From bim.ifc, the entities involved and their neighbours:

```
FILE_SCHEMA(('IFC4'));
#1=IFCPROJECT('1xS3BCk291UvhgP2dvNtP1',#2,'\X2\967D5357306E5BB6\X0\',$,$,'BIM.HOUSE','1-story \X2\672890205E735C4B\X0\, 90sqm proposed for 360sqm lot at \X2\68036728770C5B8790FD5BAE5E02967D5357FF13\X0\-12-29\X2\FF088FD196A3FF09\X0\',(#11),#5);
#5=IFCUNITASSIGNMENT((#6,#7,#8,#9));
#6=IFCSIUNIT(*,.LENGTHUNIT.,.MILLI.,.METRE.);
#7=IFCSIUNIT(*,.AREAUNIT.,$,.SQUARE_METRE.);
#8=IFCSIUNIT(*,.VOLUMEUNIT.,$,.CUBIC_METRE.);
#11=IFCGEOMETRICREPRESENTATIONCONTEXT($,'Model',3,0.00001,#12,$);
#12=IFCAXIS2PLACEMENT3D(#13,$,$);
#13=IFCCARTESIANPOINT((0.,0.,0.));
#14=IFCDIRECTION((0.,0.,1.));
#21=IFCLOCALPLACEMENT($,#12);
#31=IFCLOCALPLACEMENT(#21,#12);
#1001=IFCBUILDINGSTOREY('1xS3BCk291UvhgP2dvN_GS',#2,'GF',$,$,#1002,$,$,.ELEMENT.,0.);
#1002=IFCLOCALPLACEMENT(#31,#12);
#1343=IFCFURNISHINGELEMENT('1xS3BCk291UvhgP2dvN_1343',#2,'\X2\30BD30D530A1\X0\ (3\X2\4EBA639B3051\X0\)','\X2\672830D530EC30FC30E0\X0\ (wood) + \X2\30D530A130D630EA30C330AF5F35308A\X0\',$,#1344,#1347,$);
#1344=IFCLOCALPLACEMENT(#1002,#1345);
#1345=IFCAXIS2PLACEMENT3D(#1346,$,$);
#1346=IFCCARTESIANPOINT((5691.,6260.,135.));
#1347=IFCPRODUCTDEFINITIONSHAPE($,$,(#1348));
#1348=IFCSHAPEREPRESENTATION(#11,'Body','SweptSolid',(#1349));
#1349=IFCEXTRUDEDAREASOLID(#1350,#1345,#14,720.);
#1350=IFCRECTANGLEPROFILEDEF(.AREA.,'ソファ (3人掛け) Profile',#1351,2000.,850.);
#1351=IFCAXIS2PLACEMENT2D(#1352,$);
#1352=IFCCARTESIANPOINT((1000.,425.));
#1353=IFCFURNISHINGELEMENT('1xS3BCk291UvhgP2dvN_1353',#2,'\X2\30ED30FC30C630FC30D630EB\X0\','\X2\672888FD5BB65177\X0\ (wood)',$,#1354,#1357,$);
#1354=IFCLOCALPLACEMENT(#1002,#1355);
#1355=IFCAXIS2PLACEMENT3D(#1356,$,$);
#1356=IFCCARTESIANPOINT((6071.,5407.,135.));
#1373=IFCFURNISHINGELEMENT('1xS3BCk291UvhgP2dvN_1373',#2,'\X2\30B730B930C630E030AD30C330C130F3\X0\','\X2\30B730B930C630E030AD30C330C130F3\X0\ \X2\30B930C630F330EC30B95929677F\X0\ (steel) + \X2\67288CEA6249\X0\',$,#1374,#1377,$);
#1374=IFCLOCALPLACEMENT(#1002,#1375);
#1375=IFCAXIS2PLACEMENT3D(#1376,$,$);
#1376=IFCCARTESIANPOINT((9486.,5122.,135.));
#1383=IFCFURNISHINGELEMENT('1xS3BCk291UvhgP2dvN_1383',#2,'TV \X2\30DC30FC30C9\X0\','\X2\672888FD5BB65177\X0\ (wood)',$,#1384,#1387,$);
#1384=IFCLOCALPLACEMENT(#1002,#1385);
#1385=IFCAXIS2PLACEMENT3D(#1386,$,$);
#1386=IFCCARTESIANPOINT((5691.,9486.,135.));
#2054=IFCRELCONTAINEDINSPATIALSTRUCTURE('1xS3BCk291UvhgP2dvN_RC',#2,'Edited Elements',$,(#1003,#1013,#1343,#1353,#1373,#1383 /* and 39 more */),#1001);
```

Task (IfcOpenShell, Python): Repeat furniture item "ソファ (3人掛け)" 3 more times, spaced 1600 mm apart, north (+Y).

```python
import numpy as np
import ifcopenshell
import ifcopenshell.api.geometry
import ifcopenshell.api.root
import ifcopenshell.util.element
import ifcopenshell.util.placement
import ifcopenshell.util.unit

model = ifcopenshell.open("bim.ifc")
unit_scale = ifcopenshell.util.unit.calculate_unit_scale(model)


def reuse_history(source, copy):
    """copy_class also copies each property set's owner history, people and application; keep the originals."""
    for rel in copy.IsDefinedBy:
        if rel.is_a("IfcRelDefinesByProperties") and (history := rel.RelatingPropertyDefinition.OwnerHistory):
            rel.RelatingPropertyDefinition.OwnerHistory = source.OwnerHistory
            ifcopenshell.util.element.remove_deep2(model, history)


source = model.by_guid("1xS3BCk291UvhgP2dvN_1343")
base = ifcopenshell.util.placement.get_local_placement(source.ObjectPlacement)
step = np.array([0.0, 1.0, 0.0]) * 1.6 / unit_scale

for i in range(1, 4):
    copy = ifcopenshell.api.root.copy_class(model, product=source)
    copy.Representation = ifcopenshell.util.element.copy_deep(
        model, source.Representation, exclude=["IfcGeometricRepresentationContext", "IfcRepresentationMap"]
    )
    reuse_history(source, copy)
    matrix = base.copy()
    matrix[:3, 3] += i * step
    print("added at", matrix[:3, 3].round(3) + 0.0)
    ifcopenshell.api.geometry.edit_object_placement(model, product=copy, matrix=matrix, is_si=False)

model.write("bim_v2.ifc")
```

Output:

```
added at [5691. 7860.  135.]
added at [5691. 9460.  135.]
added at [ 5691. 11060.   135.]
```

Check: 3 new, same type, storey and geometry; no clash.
